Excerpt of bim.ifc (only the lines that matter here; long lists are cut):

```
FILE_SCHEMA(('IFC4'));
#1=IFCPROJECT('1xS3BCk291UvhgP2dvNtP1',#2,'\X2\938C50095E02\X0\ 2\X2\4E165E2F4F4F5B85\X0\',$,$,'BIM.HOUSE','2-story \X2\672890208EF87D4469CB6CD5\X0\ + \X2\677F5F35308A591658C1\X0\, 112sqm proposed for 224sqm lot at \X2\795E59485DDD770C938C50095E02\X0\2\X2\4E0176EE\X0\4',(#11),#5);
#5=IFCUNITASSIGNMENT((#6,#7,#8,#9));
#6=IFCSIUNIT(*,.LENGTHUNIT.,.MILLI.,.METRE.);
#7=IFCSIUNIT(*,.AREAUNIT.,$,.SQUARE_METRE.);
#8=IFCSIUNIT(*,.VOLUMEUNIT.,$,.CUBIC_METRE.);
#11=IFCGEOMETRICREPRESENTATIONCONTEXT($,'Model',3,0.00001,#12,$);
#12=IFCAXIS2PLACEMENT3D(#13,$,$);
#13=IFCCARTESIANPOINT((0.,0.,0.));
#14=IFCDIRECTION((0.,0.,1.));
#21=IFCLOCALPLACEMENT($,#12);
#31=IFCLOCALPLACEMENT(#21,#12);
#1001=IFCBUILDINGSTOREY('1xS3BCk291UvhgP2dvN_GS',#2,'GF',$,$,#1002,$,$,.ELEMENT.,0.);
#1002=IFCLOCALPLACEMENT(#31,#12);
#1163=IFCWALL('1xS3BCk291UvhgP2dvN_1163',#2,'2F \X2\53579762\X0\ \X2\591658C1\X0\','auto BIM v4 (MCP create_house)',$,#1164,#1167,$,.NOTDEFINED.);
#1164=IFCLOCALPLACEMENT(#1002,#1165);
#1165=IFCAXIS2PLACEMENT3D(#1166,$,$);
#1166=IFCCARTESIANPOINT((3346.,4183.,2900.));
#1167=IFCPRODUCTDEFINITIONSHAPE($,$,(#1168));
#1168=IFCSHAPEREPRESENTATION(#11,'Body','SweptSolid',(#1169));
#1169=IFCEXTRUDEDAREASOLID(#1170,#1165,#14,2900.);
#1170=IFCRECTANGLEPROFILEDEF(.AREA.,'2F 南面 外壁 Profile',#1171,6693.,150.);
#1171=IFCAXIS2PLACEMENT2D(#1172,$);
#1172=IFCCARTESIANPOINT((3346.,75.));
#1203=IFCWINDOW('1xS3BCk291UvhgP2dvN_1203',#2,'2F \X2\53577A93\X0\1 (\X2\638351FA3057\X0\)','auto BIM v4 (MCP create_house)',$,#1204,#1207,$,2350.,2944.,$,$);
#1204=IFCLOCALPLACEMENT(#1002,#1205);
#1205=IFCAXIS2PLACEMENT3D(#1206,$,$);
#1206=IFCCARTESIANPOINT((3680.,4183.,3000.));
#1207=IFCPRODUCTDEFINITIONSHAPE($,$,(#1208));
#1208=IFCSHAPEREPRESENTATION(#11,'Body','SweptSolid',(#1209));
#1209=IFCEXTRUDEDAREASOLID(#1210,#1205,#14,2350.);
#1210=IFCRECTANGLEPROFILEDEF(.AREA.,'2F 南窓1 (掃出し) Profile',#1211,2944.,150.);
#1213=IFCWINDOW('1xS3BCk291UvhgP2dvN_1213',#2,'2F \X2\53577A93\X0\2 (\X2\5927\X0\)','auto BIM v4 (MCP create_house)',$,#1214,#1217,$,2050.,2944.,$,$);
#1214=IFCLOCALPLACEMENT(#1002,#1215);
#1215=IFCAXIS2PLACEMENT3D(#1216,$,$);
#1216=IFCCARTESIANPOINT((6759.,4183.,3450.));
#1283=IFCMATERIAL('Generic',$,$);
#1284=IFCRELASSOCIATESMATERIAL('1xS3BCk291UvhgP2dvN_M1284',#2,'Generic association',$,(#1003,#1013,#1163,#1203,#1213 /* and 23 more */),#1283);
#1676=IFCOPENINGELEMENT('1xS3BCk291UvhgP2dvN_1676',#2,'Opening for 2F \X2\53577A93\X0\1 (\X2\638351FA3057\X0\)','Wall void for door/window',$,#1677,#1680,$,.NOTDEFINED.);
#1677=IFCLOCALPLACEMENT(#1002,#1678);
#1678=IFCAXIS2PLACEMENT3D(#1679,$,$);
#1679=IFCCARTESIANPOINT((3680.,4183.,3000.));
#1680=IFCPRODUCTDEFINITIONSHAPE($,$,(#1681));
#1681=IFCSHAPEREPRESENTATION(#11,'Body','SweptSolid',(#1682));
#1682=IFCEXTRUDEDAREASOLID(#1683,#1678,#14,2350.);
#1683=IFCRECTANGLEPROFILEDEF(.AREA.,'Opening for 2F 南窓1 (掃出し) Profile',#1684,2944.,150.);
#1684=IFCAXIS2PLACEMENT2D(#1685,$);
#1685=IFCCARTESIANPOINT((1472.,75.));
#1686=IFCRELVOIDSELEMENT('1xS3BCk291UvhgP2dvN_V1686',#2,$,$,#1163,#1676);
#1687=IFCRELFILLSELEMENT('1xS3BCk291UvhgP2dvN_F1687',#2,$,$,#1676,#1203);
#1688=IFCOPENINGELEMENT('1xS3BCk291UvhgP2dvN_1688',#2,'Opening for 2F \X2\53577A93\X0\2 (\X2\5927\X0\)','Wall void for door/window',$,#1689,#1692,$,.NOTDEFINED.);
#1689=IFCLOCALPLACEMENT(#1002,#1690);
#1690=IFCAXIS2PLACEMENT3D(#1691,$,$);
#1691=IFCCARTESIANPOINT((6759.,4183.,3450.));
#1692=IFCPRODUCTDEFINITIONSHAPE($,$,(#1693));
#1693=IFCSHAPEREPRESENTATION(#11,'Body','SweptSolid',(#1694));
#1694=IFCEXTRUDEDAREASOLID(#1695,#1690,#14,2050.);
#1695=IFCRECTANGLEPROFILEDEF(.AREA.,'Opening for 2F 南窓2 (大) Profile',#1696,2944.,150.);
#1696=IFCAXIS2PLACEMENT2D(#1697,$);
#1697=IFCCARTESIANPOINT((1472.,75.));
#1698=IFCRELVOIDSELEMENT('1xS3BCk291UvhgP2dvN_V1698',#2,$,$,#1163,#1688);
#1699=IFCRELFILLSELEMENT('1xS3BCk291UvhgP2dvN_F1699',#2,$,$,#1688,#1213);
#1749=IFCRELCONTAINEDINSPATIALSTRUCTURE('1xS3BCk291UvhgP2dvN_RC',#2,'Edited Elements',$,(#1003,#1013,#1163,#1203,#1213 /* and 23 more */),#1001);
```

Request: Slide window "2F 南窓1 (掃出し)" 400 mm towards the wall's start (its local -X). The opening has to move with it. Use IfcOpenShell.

```python
import ifcopenshell
import ifcopenshell.api.geometry
import ifcopenshell.util.placement
import ifcopenshell.util.unit

model = ifcopenshell.open("bim.ifc")
unit_scale = ifcopenshell.util.unit.calculate_unit_scale(model)

window = model.by_id(1203)
opening = window.FillsVoids[0].RelatingOpeningElement
wall = opening.VoidsElements[0].RelatingBuildingElement

wall_matrix = ifcopenshell.util.placement.get_local_placement(wall.ObjectPlacement)
shift = wall_matrix[:3, 0] * -0.4 / unit_scale
before = ifcopenshell.util.placement.get_local_placement(window.ObjectPlacement)[:3, 3].copy()

# The window is not placed relative to its opening, so move both.
for product in (opening, window):
    matrix = ifcopenshell.util.placement.get_local_placement(product.ObjectPlacement)
    matrix[:3, 3] += shift
    ifcopenshell.api.geometry.edit_object_placement(model, product=product, matrix=matrix, is_si=False)

after = ifcopenshell.util.placement.get_local_placement(window.ObjectPlacement)[:3, 3]
print("window moved by", (after - before).round(3) + 0.0)

model.write("bim-out.ifc")
```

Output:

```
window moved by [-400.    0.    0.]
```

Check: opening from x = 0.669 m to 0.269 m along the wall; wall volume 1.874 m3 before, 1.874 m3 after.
